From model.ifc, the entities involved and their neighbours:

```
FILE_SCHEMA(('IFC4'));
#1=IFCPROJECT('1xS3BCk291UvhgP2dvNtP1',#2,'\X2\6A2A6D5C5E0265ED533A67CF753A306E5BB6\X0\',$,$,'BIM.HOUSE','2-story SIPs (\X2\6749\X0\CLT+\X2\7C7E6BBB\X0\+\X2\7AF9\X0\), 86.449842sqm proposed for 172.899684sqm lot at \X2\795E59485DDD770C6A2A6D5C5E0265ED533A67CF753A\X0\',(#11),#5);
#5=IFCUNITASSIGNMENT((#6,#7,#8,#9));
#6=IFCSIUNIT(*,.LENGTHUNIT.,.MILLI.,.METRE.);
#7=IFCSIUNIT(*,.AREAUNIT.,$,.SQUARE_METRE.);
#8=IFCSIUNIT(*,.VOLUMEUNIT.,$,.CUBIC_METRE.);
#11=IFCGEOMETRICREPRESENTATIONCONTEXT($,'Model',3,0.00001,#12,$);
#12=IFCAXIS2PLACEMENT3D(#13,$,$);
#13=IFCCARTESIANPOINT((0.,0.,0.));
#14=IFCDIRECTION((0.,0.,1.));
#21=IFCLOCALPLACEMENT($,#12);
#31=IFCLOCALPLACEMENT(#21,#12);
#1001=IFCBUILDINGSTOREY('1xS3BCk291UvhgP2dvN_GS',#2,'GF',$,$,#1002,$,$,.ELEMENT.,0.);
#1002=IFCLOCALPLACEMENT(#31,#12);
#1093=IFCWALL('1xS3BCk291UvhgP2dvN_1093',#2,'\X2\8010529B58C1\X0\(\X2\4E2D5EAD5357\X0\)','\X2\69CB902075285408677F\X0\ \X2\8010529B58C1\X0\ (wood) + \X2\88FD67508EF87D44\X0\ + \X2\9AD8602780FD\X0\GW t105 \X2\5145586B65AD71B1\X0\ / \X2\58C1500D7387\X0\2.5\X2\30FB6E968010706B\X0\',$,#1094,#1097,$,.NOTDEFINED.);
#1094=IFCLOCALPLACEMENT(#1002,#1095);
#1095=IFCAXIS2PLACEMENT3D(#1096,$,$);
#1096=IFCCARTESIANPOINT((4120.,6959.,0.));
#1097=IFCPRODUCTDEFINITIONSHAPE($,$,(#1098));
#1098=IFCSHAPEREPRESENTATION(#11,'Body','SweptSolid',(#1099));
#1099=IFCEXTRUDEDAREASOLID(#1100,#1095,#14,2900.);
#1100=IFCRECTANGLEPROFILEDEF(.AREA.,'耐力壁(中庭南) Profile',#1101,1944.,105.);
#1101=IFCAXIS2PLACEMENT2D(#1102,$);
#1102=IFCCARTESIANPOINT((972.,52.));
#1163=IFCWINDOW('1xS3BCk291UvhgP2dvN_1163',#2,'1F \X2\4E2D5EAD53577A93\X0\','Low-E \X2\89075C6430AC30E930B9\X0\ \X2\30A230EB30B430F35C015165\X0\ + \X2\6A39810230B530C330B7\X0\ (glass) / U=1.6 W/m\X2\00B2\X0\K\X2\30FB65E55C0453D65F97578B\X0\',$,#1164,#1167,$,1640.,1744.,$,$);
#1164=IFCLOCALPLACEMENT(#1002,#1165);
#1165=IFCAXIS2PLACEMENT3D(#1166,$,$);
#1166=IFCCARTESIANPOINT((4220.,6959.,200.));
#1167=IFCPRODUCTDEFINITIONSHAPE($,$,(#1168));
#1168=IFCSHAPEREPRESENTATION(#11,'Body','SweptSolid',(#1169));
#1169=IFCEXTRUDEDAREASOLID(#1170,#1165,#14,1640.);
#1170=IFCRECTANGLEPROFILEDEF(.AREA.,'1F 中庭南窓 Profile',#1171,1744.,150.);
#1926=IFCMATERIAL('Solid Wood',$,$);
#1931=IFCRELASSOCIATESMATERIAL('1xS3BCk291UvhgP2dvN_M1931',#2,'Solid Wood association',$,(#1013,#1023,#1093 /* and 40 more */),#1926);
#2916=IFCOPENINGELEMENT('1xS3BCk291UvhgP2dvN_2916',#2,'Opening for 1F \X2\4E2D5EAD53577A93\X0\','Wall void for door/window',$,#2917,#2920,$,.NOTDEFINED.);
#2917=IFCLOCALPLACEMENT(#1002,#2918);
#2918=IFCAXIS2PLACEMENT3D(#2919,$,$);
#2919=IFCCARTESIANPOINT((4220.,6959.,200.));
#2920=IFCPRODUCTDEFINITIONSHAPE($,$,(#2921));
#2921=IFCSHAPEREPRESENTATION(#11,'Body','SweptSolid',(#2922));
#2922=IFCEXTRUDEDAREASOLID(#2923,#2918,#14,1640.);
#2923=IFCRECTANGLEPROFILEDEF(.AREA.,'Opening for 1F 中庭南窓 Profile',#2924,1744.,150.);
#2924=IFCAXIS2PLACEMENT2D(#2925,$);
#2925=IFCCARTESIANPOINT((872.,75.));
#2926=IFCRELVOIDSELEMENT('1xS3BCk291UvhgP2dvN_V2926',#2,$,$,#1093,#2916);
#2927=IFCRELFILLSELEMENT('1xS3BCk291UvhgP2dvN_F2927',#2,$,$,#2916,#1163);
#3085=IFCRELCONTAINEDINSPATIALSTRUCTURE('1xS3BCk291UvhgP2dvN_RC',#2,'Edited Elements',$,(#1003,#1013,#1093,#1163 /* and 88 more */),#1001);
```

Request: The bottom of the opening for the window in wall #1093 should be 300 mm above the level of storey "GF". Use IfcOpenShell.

```python
import numpy as np
import ifcopenshell
import ifcopenshell.api.geometry
import ifcopenshell.geom
import ifcopenshell.util.element
import ifcopenshell.util.placement
import ifcopenshell.util.shape
import ifcopenshell.util.unit

model = ifcopenshell.open("model.ifc")
unit_scale = ifcopenshell.util.unit.calculate_unit_scale(model)

window = model.by_guid("1xS3BCk291UvhgP2dvN_1163")
opening = window.FillsVoids[0].RelatingOpeningElement
storey = ifcopenshell.util.element.get_container(window, ifc_class="IfcBuildingStorey")
level = ifcopenshell.util.placement.get_local_placement(storey.ObjectPlacement)[2, 3]

# The opening's origin need not be at the sill, so measure its lowest point.
shape = ifcopenshell.geom.create_shape(ifcopenshell.geom.settings(), opening)
bottom = ifcopenshell.util.shape.get_shape_bottom_elevation(shape, shape.geometry) / unit_scale
dz = level + 300.0 - bottom

shift = np.array([0.0, 0.0, dz])
# The window is not placed relative to its opening, so move both.
for product in (opening, window):
    matrix = ifcopenshell.util.placement.get_local_placement(product.ObjectPlacement)
    matrix[:3, 3] += shift
    ifcopenshell.api.geometry.edit_object_placement(model, product=product, matrix=matrix, is_si=False)

print(f"moved by {dz * unit_scale:+.3f} m")

model.write("model_v2.ifc")
```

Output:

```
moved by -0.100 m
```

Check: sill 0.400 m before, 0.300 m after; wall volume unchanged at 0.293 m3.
